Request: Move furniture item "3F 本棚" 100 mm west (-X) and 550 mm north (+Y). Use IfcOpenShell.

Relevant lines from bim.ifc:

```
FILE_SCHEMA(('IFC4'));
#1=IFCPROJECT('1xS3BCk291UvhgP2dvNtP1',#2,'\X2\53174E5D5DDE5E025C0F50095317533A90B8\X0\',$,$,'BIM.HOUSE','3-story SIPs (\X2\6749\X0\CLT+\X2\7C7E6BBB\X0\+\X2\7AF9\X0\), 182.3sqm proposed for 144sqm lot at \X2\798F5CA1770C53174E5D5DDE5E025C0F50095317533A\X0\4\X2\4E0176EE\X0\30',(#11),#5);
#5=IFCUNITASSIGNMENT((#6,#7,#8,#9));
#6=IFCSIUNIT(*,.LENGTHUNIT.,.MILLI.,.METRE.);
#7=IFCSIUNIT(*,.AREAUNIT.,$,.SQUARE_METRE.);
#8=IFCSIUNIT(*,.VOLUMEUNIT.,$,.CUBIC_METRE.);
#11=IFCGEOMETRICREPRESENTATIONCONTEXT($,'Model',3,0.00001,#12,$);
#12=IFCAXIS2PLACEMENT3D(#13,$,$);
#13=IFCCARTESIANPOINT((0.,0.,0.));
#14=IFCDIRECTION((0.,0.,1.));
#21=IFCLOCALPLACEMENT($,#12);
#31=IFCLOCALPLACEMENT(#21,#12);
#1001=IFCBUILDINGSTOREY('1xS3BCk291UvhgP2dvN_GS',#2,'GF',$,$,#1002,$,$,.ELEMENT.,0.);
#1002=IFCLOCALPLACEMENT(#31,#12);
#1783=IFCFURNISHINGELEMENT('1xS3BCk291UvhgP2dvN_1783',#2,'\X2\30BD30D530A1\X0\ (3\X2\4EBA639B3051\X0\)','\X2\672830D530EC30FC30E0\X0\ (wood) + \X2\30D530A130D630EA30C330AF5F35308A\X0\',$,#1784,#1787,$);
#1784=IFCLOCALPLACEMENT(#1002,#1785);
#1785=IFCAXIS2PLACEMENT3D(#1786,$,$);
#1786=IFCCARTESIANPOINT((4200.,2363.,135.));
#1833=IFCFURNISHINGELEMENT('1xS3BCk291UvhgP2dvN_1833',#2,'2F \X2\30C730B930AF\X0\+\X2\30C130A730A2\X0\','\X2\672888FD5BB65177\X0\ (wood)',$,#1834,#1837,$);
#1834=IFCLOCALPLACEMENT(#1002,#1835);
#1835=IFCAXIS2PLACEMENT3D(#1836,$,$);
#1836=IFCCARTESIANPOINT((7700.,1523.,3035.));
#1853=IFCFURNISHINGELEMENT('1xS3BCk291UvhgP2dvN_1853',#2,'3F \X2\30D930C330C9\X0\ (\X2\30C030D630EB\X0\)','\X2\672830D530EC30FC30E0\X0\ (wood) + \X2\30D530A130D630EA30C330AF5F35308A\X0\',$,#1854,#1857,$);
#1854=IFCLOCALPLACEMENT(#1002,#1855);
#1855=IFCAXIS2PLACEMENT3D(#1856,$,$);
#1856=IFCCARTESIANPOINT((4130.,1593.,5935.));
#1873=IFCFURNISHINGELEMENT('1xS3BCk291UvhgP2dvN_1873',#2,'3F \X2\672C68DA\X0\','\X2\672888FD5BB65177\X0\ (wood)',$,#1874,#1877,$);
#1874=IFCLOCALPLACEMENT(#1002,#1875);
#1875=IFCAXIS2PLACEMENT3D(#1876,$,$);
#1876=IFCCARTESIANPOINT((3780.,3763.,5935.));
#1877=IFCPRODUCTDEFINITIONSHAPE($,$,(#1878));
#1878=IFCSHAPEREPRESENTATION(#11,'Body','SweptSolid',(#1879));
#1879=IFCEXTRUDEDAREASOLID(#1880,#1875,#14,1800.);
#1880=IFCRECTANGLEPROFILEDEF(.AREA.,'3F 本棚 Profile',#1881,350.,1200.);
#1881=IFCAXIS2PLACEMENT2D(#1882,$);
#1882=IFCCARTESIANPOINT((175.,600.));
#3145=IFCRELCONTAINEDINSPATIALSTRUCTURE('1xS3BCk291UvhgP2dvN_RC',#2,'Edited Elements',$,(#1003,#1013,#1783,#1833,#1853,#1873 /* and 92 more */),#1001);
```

```python
import ifcopenshell
import ifcopenshell.api.geometry
import ifcopenshell.util.placement
import ifcopenshell.util.unit

model = ifcopenshell.open("bim.ifc")
unit_scale = ifcopenshell.util.unit.calculate_unit_scale(model)

item = model.by_guid("1xS3BCk291UvhgP2dvN_1873")
matrix = ifcopenshell.util.placement.get_local_placement(item.ObjectPlacement)
matrix[0, 3] -= 0.1 / unit_scale
matrix[1, 3] += 0.55 / unit_scale
ifcopenshell.api.geometry.edit_object_placement(model, product=item, matrix=matrix, is_si=False)

print(ifcopenshell.util.placement.get_local_placement(item.ObjectPlacement).round(3) + 0.0)

model.write("bim-out.ifc")
```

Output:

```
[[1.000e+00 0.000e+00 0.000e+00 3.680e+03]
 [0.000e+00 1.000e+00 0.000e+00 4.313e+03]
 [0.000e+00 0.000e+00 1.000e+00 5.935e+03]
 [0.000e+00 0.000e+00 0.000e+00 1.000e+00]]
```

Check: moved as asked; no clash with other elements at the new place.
